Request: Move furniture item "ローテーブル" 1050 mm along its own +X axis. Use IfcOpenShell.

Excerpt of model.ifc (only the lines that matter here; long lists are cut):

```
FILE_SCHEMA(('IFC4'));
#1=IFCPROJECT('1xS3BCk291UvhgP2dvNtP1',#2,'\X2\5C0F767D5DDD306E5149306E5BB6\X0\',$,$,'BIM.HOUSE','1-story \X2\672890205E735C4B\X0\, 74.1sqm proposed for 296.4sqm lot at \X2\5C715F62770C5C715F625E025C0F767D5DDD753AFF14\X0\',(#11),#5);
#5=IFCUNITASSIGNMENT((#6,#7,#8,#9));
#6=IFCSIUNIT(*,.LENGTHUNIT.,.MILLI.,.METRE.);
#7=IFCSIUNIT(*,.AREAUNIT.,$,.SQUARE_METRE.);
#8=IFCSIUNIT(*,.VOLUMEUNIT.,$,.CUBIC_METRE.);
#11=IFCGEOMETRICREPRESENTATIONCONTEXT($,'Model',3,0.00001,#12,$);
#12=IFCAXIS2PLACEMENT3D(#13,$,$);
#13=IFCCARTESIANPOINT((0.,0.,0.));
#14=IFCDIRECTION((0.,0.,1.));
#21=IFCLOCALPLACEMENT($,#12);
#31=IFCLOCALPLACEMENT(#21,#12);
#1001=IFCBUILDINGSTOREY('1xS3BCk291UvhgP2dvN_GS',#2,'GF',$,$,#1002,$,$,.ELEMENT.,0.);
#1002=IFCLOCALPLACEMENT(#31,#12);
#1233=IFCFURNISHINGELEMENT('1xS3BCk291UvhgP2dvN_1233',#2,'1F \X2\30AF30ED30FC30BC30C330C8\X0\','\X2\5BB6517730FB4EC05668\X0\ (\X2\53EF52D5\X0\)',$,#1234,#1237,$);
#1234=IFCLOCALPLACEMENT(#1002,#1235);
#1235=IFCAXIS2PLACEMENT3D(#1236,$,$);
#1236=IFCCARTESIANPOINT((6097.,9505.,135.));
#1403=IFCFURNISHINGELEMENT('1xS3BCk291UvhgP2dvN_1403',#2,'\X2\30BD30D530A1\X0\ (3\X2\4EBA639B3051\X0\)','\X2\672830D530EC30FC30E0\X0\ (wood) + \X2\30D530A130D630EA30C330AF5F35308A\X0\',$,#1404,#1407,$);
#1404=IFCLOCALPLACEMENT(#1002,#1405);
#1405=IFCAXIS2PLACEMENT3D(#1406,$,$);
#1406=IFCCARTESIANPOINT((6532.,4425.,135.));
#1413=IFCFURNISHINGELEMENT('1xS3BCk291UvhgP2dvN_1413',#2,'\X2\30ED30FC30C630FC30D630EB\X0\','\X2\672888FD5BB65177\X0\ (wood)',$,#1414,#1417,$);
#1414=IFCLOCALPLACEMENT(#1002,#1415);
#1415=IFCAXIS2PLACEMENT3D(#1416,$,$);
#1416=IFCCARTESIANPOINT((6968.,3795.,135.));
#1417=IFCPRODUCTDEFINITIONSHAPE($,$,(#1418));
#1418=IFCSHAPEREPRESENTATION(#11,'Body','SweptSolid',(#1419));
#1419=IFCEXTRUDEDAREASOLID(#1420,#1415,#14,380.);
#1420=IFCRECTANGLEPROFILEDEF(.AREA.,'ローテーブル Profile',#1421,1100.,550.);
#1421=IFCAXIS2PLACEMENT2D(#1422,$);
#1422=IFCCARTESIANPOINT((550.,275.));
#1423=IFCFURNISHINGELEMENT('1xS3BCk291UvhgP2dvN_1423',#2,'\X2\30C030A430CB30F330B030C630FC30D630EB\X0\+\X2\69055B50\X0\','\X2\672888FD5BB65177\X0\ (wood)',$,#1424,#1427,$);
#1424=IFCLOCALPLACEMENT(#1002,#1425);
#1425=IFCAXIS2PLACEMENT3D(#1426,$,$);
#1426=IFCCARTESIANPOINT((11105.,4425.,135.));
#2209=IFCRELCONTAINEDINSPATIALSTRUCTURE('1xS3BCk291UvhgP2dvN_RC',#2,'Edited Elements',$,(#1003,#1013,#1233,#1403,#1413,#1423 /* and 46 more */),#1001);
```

```python
import ifcopenshell
import ifcopenshell.api.geometry
import ifcopenshell.util.placement
import ifcopenshell.util.unit

model = ifcopenshell.open("model.ifc")
unit_scale = ifcopenshell.util.unit.calculate_unit_scale(model)

item = model.by_guid("1xS3BCk291UvhgP2dvN_1413")
matrix = ifcopenshell.util.placement.get_local_placement(item.ObjectPlacement)
matrix[:3, 3] += matrix[:3, 0] * 1.05 / unit_scale
ifcopenshell.api.geometry.edit_object_placement(model, product=item, matrix=matrix, is_si=False)

print(ifcopenshell.util.placement.get_local_placement(item.ObjectPlacement).round(3) + 0.0)

model.write("model_rev.ifc")
```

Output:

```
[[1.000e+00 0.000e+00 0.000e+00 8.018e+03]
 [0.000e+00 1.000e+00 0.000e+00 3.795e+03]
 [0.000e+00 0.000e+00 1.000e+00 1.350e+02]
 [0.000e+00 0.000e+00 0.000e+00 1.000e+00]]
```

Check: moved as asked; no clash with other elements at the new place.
